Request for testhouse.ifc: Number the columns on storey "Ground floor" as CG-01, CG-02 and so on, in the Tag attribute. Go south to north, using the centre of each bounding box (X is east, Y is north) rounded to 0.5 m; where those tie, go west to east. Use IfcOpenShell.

First a look at what the model holds.

```python
import ifcopenshell
import ifcopenshell.util.element
import ifcopenshell.util.placement

model = ifcopenshell.open("testhouse.ifc")
print(model.schema)
storey = next(s for s in model.by_type("IfcBuildingStorey") if s.Name == "Ground floor")
columns = [e for e in ifcopenshell.util.element.get_decomposition(storey) if e.is_a("IfcColumn")]
for e in sorted(columns, key=lambda e: e.id()):
    origin = ifcopenshell.util.placement.get_local_placement(e.ObjectPlacement)[:3, 3]
    print(e.id(), e.Tag, e.Name, origin.round(2) + 0.0, sep=" | ")
```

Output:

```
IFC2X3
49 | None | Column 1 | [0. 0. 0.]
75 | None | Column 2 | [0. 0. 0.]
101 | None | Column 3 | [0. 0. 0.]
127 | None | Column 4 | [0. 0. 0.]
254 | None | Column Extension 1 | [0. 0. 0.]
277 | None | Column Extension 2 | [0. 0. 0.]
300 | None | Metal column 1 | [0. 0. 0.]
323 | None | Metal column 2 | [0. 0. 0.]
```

```python
import ifcopenshell
import ifcopenshell.geom
import ifcopenshell.util.element
import ifcopenshell.util.shape

model = ifcopenshell.open("testhouse.ifc")
settings = ifcopenshell.geom.settings()
settings.set("use-world-coords", True)


def centre(element):
    shape = ifcopenshell.geom.create_shape(settings, element)
    return ifcopenshell.util.shape.get_bbox_centroid(shape.geometry)


storey = next(s for s in model.by_type("IfcBuildingStorey") if s.Name == "Ground floor")
columns = [e for e in ifcopenshell.util.element.get_decomposition(storey) if e.is_a("IfcColumn")]

# Insertion points can sit at a corner or the storey origin, so sort by the geometry (in metres).
centres = {e: centre(e) for e in columns}
columns.sort(key=lambda e: (round(centres[e][1] / 0.5), centres[e][0]))

for i, e in enumerate(columns, start=1):
    number = f"CG-{i:02d}"
    e.Tag = number
    print(e.id(), number)

model.write("testhouse-out.ifc")
```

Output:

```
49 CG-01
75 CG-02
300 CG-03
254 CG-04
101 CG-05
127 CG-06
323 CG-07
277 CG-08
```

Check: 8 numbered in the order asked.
